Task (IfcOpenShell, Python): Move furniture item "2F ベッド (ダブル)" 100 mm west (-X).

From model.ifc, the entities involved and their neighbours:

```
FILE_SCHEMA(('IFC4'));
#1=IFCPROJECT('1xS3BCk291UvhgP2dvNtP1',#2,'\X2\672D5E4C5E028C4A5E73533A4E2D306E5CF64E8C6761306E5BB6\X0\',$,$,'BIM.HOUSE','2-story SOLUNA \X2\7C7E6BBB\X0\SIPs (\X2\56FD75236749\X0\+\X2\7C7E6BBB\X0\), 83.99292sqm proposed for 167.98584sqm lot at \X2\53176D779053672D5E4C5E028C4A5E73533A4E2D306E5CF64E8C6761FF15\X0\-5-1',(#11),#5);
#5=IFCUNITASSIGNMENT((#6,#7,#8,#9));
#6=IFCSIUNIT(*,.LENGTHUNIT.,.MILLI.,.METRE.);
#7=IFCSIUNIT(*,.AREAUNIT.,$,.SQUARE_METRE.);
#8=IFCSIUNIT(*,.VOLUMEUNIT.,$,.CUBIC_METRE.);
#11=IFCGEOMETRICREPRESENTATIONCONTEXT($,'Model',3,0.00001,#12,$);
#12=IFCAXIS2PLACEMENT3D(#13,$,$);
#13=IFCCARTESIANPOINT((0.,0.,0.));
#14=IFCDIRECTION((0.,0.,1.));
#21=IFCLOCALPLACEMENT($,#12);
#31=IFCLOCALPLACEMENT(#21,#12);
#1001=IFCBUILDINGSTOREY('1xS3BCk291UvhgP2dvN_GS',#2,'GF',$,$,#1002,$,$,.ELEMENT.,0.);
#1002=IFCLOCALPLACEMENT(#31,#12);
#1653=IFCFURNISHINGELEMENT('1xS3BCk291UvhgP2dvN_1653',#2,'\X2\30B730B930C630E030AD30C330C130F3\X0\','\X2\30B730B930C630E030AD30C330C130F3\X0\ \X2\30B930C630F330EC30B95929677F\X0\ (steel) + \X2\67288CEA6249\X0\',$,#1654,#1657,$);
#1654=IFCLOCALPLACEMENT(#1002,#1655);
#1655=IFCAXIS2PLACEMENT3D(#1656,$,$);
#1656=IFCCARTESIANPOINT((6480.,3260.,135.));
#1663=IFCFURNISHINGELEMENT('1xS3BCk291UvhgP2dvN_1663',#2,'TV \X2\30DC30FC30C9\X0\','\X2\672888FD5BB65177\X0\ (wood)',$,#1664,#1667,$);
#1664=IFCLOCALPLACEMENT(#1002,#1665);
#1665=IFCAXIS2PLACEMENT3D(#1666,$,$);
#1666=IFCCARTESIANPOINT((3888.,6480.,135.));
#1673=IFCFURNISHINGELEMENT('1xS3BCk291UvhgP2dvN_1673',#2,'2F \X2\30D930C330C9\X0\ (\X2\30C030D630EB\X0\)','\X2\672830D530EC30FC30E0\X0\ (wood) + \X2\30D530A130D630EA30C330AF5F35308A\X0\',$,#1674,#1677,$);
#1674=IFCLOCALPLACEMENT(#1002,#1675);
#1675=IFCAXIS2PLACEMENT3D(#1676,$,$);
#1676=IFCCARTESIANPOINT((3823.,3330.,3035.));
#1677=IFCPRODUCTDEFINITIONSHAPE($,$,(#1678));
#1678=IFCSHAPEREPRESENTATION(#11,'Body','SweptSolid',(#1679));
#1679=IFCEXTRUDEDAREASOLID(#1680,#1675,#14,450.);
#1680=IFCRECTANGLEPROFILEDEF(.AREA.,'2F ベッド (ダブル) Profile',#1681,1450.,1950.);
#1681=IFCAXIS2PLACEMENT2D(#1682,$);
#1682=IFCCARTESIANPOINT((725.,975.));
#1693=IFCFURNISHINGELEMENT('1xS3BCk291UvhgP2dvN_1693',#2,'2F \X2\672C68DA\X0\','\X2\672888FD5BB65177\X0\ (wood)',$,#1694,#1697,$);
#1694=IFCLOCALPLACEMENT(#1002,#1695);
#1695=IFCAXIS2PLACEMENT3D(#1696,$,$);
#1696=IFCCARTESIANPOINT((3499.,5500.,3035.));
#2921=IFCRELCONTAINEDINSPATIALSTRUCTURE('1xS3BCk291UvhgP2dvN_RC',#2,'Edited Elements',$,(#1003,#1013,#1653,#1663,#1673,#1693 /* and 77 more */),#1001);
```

```python
import ifcopenshell
import ifcopenshell.api.geometry
import ifcopenshell.util.placement
import ifcopenshell.util.unit

model = ifcopenshell.open("model.ifc")
unit_scale = ifcopenshell.util.unit.calculate_unit_scale(model)

item = model.by_id(1673)
matrix = ifcopenshell.util.placement.get_local_placement(item.ObjectPlacement)
matrix[0, 3] -= 0.1 / unit_scale
ifcopenshell.api.geometry.edit_object_placement(model, product=item, matrix=matrix, is_si=False)

print(ifcopenshell.util.placement.get_local_placement(item.ObjectPlacement).round(3) + 0.0)

model.write("model_edited.ifc")
```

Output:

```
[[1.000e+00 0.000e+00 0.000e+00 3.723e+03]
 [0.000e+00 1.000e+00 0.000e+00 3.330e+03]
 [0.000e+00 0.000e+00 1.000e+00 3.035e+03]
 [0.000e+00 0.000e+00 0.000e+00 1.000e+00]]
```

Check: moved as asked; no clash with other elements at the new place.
